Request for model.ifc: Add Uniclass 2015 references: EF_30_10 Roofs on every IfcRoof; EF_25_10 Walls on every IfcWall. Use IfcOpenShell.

First a look at what the model holds.

```python
import ifcopenshell

model = ifcopenshell.open("model.ifc")
print(model.schema)
print("classifications:", [c.Name for c in model.by_type("IfcClassification")])
for ifc_class in ("IfcDoor", "IfcRoof", "IfcStair", "IfcWall", "IfcWindow"):
    print(ifc_class, len(model.by_type(ifc_class)))
```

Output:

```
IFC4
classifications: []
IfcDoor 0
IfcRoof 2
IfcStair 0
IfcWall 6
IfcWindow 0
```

```python
import ifcopenshell
import ifcopenshell.api.classification

model = ifcopenshell.open("model.ifc")

system = ifcopenshell.api.classification.add_classification(model, classification="Uniclass 2015")

codes = {
    "IfcRoof": ("EF_30_10", "Roofs"),
    "IfcWall": ("EF_25_10", "Walls"),
}
for ifc_class, (code, name) in codes.items():
    products = model.by_type(ifc_class)
    ifcopenshell.api.classification.add_reference(
        model, products=products, classification=system, identification=code, name=name
    )
    print(code, len(products))

model.write("model-out.ifc")
```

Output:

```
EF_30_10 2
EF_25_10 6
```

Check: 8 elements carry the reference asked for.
